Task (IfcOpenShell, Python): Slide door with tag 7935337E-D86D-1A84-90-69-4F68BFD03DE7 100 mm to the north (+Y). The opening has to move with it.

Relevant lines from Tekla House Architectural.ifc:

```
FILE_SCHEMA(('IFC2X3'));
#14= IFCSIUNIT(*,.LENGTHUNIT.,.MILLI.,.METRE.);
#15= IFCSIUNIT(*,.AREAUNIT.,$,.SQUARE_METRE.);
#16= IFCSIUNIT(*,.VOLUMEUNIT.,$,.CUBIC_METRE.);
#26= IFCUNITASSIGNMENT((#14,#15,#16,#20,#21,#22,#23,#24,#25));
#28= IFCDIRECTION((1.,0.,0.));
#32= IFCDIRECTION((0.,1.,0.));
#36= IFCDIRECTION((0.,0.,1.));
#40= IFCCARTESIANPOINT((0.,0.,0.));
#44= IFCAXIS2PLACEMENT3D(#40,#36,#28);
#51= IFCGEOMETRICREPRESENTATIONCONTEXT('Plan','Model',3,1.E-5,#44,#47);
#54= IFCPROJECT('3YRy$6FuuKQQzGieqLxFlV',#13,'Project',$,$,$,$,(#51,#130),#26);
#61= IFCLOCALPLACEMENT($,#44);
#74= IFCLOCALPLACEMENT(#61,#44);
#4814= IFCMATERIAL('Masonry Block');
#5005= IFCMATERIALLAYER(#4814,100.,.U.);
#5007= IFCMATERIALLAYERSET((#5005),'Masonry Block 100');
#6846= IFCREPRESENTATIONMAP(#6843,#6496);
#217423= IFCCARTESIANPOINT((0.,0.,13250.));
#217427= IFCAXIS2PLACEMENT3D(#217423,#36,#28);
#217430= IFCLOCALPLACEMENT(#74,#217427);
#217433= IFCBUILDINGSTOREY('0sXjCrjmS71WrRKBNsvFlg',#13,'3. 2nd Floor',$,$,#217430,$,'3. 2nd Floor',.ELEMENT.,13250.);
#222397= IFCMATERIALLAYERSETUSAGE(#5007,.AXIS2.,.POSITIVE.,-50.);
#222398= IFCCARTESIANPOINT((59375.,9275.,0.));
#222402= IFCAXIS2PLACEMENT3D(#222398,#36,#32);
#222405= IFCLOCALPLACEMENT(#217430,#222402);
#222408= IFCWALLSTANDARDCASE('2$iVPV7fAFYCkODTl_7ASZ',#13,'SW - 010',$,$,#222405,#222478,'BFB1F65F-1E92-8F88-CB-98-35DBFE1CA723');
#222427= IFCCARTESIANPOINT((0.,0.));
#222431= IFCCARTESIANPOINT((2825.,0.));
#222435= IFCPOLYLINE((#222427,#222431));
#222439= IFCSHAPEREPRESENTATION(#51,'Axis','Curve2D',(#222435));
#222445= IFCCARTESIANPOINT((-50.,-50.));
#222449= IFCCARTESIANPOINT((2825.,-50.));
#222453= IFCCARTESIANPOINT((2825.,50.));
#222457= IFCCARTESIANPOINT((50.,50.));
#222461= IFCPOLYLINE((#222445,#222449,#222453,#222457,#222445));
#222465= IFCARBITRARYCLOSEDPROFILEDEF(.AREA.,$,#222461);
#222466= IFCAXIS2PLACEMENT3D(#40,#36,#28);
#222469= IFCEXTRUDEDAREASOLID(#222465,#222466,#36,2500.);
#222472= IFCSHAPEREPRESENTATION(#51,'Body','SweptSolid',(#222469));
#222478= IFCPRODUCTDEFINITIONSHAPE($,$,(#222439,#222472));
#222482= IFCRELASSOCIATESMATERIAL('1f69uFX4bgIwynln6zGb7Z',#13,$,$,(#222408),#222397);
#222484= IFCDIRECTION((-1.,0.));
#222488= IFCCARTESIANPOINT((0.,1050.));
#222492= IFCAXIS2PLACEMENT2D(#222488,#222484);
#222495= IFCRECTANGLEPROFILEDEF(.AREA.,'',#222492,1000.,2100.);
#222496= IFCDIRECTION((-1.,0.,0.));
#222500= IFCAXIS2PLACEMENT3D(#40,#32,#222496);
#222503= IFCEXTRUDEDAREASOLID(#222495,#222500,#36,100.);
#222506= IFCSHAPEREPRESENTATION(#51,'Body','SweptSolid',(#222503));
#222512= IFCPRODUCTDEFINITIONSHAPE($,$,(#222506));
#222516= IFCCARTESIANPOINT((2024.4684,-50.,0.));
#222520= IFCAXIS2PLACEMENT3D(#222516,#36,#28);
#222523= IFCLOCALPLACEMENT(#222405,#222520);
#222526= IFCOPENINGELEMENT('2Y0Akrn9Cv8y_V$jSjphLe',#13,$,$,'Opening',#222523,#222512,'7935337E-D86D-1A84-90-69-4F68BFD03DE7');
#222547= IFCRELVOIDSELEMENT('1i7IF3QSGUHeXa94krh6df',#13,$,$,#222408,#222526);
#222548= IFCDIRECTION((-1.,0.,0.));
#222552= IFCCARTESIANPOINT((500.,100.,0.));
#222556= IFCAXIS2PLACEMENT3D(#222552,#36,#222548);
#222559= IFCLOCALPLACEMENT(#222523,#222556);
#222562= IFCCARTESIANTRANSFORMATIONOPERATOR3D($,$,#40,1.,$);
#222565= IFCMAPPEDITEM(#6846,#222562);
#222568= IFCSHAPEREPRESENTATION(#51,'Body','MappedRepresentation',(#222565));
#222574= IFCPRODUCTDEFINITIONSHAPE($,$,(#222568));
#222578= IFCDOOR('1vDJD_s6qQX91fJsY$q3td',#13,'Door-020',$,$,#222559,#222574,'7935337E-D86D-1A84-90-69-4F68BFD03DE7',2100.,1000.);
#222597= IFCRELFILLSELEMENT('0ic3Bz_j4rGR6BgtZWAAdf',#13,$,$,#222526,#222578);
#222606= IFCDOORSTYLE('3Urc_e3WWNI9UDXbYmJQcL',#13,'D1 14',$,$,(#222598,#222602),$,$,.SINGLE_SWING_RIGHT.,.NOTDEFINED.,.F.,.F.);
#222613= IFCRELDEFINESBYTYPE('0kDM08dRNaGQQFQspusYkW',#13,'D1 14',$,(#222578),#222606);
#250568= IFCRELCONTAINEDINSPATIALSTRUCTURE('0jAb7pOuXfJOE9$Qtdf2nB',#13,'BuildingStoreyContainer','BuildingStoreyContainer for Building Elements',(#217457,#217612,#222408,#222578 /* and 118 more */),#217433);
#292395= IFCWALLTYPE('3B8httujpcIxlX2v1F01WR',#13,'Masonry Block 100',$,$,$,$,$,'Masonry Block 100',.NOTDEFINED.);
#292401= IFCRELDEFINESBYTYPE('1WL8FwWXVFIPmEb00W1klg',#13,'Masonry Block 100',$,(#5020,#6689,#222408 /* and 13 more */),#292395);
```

```python
import ifcopenshell
import ifcopenshell.api.geometry
import ifcopenshell.util.placement
import ifcopenshell.util.unit

model = ifcopenshell.open("Tekla House Architectural.ifc")
unit_scale = ifcopenshell.util.unit.calculate_unit_scale(model)

door = model.by_guid("1vDJD_s6qQX91fJsY$q3td")
opening = door.FillsVoids[0].RelatingOpeningElement
wall = opening.VoidsElements[0].RelatingBuildingElement

wall_matrix = ifcopenshell.util.placement.get_local_placement(wall.ObjectPlacement)
shift = wall_matrix[:3, 0] * 0.1 / unit_scale
before = ifcopenshell.util.placement.get_local_placement(door.ObjectPlacement)[:3, 3].copy()

# The door is placed relative to its opening, so it follows when the opening moves.
matrix = ifcopenshell.util.placement.get_local_placement(opening.ObjectPlacement)
matrix[:3, 3] += shift
ifcopenshell.api.geometry.edit_object_placement(
    model, product=opening, matrix=matrix, is_si=False, should_transform_children=True
)

after = ifcopenshell.util.placement.get_local_placement(door.ObjectPlacement)[:3, 3]
print("door moved by", (after - before).round(3) + 0.0)

model.write("Tekla House Architectural_edited.ifc")
```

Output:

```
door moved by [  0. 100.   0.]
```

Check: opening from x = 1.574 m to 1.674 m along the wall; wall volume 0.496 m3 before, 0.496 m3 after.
